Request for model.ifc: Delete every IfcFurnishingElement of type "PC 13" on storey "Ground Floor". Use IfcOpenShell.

First a look at what the model holds.

```python
import ifcopenshell
import ifcopenshell.util.element

model = ifcopenshell.open("model.ifc")
print(model.schema)
storey = next(s for s in model.by_type("IfcBuildingStorey") if s.Name == "Ground Floor")
furniture = [e for e in ifcopenshell.util.element.get_decomposition(storey) if e.is_a("IfcFurnishingElement")]
seen = {}
for e in furniture:
    element_type = ifcopenshell.util.element.get_type(e)
    name = element_type.Name if element_type not in (None, e) else None
    seen[name] = seen.get(name, 0) + 1
for name, count in sorted(seen.items(), key=str):
    print(count, "x", name)
```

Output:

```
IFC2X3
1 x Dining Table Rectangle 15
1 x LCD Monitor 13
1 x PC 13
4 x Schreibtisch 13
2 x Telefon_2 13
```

```python
import ifcopenshell
import ifcopenshell.api.root
import ifcopenshell.util.element

model = ifcopenshell.open("model.ifc")

storey = next(s for s in model.by_type("IfcBuildingStorey") if s.Name == "Ground Floor")
furniture = [e for e in ifcopenshell.util.element.get_decomposition(storey) if e.is_a("IfcFurnishingElement")]
targets = [e for e in furniture if (t := ifcopenshell.util.element.get_type(e)) not in (None, e) and t.Name == "PC 13"]

for e in targets:
    ifcopenshell.api.root.remove_product(model, product=e)
print(len(targets), "removed")

model.write("model_v2.ifc")
```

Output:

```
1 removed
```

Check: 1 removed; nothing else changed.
